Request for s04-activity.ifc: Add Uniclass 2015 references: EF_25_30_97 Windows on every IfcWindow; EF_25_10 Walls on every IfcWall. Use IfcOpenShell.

First a look at what the model holds.

```python
import ifcopenshell

model = ifcopenshell.open("s04-activity.ifc")
print(model.schema)
print("classifications:", [c.Name for c in model.by_type("IfcClassification")])
for ifc_class in ("IfcDoor", "IfcRoof", "IfcStair", "IfcWall", "IfcWindow"):
    print(ifc_class, len(model.by_type(ifc_class)))
```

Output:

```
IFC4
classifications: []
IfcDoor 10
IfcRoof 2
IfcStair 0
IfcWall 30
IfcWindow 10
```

```python
import ifcopenshell
import ifcopenshell.api.classification

model = ifcopenshell.open("s04-activity.ifc")

system = ifcopenshell.api.classification.add_classification(model, classification="Uniclass 2015")

codes = {
    "IfcWindow": ("EF_25_30_97", "Windows"),
    "IfcWall": ("EF_25_10", "Walls"),
}
for ifc_class, (code, name) in codes.items():
    products = model.by_type(ifc_class)
    ifcopenshell.api.classification.add_reference(
        model, products=products, classification=system, identification=code, name=name
    )
    print(code, len(products))

model.write("s04-activity_v2.ifc")
```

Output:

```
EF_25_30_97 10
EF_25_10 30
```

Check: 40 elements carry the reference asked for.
